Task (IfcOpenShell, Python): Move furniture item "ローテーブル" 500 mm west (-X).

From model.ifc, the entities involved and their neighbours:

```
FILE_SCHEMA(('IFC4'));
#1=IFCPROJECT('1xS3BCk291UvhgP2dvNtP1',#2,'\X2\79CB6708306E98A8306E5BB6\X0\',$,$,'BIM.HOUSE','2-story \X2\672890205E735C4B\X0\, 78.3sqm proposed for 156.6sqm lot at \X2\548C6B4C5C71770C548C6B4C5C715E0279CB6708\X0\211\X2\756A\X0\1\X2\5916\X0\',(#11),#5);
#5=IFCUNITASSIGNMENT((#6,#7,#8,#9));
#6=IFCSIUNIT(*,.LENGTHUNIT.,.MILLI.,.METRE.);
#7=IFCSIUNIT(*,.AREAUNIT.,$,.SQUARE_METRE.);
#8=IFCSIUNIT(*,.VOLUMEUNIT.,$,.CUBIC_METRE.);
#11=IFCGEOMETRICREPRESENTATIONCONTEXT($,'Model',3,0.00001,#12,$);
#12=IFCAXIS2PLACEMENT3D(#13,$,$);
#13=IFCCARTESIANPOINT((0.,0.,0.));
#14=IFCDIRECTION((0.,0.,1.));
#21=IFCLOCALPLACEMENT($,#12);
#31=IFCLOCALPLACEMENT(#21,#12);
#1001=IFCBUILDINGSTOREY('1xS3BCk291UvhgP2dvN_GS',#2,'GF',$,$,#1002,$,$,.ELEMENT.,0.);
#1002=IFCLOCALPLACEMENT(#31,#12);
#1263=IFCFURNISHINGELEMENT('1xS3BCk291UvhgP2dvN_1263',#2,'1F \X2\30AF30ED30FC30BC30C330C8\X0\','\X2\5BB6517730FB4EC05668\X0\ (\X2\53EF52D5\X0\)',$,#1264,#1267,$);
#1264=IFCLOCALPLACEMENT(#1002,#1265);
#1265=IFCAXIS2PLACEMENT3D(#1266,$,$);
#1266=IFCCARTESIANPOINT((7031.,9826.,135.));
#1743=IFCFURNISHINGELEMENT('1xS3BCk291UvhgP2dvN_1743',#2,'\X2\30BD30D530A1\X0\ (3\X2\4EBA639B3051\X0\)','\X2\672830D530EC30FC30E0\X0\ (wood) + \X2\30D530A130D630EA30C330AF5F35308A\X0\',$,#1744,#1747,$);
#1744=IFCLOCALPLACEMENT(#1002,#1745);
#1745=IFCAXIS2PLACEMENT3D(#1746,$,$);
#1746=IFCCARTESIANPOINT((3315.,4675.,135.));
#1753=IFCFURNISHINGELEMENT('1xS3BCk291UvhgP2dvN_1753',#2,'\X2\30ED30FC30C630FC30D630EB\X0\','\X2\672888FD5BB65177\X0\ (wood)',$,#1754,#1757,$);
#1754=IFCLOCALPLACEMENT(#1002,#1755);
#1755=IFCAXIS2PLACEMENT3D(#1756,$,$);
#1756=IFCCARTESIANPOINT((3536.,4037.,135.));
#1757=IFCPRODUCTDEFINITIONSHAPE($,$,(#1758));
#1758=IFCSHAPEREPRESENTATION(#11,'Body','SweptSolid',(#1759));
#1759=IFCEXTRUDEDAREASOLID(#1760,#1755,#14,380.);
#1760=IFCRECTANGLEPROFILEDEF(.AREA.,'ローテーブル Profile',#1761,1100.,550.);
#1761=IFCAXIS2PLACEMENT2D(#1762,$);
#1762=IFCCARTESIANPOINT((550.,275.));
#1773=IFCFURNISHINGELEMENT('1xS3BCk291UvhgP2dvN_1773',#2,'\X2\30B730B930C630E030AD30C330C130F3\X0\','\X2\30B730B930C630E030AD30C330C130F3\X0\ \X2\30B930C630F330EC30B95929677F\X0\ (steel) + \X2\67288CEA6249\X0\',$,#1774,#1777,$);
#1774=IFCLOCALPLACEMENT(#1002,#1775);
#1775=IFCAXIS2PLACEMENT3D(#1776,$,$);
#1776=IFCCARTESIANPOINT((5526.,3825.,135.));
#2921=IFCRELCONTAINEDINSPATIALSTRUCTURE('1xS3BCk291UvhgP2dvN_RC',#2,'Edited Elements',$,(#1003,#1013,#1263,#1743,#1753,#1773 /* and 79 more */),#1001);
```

```python
import ifcopenshell
import ifcopenshell.api.geometry
import ifcopenshell.util.placement

model = ifcopenshell.open("model.ifc")

item = model.by_guid("1xS3BCk291UvhgP2dvN_1753")
matrix = ifcopenshell.util.placement.get_local_placement(item.ObjectPlacement)
matrix[0, 3] -= 500.0
ifcopenshell.api.geometry.edit_object_placement(model, product=item, matrix=matrix, is_si=False)

print(ifcopenshell.util.placement.get_local_placement(item.ObjectPlacement).round(3) + 0.0)

model.write("model_v2.ifc")
```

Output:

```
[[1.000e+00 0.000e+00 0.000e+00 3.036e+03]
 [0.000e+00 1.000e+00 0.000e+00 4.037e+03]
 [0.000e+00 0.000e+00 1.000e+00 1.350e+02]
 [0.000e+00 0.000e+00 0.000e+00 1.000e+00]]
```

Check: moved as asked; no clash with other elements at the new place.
